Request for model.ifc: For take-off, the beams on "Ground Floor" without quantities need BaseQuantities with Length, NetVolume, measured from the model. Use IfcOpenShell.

First a look at what the model holds.

```python
import ifcopenshell
import ifcopenshell.util.element
import ifcopenshell.util.unit

model = ifcopenshell.open("model.ifc")
print(model.schema)
for unit_type in ("LENGTHUNIT", "AREAUNIT", "VOLUMEUNIT"):
    print(unit_type, ifcopenshell.util.unit.calculate_unit_scale(model, unit_type))
storey = next(s for s in model.by_type("IfcBuildingStorey") if s.Name == "Ground Floor")
beams = [e for e in ifcopenshell.util.element.get_decomposition(storey) if e.is_a("IfcBeam")]
for e in sorted(beams, key=lambda e: e.id()):
    print(e.id(), e.is_a(), e.Name, list(ifcopenshell.util.element.get_psets(e, qtos_only=True)), sep=" | ")
```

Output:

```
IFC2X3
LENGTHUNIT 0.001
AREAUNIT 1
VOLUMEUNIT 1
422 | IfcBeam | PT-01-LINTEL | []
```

```python
import ifcopenshell
import ifcopenshell.api.pset
import ifcopenshell.geom
import ifcopenshell.util.element
import ifcopenshell.util.shape
import ifcopenshell.util.unit

model = ifcopenshell.open("model.ifc")
unit_scale = ifcopenshell.util.unit.calculate_unit_scale(model)
volume_scale = ifcopenshell.util.unit.calculate_unit_scale(model, "VOLUMEUNIT")
settings = ifcopenshell.geom.settings()

storey = next(s for s in model.by_type("IfcBuildingStorey") if s.Name == "Ground Floor")
beams = [e for e in ifcopenshell.util.element.get_decomposition(storey) if e.is_a("IfcBeam")]

for e in sorted(beams, key=lambda e: e.id()):
    if ifcopenshell.util.element.get_psets(e, qtos_only=True, should_inherit=False):
        continue
    # Geometry comes back in metres, in the element's own axes.
    shape = ifcopenshell.geom.create_shape(settings, e)
    values = {
        "Length": ifcopenshell.util.shape.get_max_xyz(shape.geometry) / unit_scale,
        "NetVolume": ifcopenshell.util.shape.get_volume(shape.geometry) / volume_scale,
    }
    qto = ifcopenshell.api.pset.add_qto(model, product=e, name="BaseQuantities")
    ifcopenshell.api.pset.edit_qto(model, qto=qto, properties=values)
    print(e.id(), {k: round(v, 3) for k, v in values.items()})

model.write("model-out.ifc")
```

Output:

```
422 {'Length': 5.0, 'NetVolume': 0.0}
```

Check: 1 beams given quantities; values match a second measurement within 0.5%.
